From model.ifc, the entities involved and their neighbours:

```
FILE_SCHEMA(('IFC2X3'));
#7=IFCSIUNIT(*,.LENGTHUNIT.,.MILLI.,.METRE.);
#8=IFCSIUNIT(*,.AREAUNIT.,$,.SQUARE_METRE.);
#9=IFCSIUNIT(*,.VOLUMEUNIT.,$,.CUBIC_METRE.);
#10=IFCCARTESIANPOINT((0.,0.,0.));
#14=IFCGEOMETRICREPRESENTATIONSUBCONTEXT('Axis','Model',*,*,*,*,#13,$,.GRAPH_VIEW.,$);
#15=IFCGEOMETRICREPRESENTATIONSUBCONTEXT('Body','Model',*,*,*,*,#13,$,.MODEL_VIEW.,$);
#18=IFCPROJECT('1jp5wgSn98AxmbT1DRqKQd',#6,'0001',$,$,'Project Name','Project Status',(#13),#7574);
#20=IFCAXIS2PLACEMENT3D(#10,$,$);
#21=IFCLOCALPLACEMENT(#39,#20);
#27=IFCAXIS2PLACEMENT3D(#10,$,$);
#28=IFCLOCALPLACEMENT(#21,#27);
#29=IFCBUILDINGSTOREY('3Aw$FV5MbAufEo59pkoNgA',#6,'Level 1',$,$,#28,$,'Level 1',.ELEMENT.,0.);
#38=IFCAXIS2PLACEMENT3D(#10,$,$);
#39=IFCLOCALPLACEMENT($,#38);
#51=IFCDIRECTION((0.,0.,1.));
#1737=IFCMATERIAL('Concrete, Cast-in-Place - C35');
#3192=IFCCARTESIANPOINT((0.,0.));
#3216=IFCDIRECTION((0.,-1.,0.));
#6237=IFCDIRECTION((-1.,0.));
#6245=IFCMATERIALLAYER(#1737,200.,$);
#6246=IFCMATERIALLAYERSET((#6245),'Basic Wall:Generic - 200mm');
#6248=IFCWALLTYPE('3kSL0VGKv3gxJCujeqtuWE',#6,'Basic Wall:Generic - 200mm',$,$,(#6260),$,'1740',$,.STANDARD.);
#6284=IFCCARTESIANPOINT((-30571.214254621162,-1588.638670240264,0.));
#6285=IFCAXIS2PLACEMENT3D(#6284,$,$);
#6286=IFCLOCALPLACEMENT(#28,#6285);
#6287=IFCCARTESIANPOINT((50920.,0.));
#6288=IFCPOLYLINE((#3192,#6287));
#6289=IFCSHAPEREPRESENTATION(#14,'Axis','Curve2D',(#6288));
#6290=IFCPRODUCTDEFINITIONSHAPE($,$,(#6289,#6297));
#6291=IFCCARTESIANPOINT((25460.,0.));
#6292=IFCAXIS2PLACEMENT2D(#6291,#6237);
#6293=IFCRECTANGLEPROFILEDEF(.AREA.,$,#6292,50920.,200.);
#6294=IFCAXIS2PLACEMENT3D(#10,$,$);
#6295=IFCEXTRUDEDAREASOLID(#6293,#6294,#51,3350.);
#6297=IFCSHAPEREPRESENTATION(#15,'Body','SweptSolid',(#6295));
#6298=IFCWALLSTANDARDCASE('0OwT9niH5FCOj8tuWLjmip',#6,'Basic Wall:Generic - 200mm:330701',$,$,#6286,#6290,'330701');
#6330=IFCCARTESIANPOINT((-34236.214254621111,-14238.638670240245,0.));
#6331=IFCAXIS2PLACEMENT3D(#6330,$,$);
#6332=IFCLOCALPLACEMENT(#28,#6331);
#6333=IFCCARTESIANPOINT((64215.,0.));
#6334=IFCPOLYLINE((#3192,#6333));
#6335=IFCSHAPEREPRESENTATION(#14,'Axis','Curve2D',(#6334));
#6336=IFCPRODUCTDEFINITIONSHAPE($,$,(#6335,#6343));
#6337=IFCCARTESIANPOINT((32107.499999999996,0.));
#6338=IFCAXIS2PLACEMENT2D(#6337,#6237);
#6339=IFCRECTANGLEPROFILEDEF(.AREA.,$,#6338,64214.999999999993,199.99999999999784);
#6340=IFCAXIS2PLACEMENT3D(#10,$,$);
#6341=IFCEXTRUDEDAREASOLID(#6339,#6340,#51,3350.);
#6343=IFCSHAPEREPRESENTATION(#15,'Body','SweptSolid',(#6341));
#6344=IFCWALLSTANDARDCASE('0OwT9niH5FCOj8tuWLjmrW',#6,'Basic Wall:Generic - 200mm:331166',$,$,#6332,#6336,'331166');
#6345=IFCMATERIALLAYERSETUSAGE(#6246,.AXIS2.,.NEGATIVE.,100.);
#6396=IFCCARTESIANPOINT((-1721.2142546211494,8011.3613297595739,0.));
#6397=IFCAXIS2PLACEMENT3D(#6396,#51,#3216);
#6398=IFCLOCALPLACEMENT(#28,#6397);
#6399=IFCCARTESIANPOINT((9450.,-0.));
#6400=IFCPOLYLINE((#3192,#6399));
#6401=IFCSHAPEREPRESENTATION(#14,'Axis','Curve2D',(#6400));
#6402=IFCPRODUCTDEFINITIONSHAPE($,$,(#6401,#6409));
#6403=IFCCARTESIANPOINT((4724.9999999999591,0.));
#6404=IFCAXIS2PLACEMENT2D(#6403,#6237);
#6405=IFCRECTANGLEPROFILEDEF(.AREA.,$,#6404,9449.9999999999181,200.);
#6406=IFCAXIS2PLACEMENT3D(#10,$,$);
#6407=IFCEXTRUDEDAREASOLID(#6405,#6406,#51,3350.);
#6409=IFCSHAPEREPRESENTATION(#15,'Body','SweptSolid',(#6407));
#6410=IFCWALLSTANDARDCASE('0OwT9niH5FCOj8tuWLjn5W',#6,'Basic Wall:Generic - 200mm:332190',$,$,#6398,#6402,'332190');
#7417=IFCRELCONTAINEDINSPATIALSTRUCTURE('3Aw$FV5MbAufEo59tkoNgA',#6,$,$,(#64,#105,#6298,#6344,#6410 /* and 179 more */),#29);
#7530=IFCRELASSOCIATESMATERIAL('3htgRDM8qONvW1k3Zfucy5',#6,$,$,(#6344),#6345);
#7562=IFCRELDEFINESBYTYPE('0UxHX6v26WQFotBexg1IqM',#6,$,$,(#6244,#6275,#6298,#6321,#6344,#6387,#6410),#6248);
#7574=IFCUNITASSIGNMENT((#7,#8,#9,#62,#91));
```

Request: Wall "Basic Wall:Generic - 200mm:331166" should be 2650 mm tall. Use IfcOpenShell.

```python
import ifcopenshell
import ifcopenshell.geom
import ifcopenshell.util.representation
import ifcopenshell.util.shape

model = ifcopenshell.open("model.ifc")
settings = ifcopenshell.geom.settings()


def volume(element):
    """Net volume in cubic metres, openings subtracted."""
    shape = ifcopenshell.geom.create_shape(settings, element)
    return ifcopenshell.util.shape.get_volume(shape.geometry)


wall = model.by_id(6344)
before = volume(wall)

body = ifcopenshell.util.representation.get_representation(wall, "Model", "Body")
solid = body.Items[0]
old_height = solid.Depth
solid.Depth = 2650.0
after = volume(wall)

print(f"height {old_height:g} -> {solid.Depth:g}, volume {before:.3f} -> {after:.3f} m3")

model.write("model_rev.ifc")
```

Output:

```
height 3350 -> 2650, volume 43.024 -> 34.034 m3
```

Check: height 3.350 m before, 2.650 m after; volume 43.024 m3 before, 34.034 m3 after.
